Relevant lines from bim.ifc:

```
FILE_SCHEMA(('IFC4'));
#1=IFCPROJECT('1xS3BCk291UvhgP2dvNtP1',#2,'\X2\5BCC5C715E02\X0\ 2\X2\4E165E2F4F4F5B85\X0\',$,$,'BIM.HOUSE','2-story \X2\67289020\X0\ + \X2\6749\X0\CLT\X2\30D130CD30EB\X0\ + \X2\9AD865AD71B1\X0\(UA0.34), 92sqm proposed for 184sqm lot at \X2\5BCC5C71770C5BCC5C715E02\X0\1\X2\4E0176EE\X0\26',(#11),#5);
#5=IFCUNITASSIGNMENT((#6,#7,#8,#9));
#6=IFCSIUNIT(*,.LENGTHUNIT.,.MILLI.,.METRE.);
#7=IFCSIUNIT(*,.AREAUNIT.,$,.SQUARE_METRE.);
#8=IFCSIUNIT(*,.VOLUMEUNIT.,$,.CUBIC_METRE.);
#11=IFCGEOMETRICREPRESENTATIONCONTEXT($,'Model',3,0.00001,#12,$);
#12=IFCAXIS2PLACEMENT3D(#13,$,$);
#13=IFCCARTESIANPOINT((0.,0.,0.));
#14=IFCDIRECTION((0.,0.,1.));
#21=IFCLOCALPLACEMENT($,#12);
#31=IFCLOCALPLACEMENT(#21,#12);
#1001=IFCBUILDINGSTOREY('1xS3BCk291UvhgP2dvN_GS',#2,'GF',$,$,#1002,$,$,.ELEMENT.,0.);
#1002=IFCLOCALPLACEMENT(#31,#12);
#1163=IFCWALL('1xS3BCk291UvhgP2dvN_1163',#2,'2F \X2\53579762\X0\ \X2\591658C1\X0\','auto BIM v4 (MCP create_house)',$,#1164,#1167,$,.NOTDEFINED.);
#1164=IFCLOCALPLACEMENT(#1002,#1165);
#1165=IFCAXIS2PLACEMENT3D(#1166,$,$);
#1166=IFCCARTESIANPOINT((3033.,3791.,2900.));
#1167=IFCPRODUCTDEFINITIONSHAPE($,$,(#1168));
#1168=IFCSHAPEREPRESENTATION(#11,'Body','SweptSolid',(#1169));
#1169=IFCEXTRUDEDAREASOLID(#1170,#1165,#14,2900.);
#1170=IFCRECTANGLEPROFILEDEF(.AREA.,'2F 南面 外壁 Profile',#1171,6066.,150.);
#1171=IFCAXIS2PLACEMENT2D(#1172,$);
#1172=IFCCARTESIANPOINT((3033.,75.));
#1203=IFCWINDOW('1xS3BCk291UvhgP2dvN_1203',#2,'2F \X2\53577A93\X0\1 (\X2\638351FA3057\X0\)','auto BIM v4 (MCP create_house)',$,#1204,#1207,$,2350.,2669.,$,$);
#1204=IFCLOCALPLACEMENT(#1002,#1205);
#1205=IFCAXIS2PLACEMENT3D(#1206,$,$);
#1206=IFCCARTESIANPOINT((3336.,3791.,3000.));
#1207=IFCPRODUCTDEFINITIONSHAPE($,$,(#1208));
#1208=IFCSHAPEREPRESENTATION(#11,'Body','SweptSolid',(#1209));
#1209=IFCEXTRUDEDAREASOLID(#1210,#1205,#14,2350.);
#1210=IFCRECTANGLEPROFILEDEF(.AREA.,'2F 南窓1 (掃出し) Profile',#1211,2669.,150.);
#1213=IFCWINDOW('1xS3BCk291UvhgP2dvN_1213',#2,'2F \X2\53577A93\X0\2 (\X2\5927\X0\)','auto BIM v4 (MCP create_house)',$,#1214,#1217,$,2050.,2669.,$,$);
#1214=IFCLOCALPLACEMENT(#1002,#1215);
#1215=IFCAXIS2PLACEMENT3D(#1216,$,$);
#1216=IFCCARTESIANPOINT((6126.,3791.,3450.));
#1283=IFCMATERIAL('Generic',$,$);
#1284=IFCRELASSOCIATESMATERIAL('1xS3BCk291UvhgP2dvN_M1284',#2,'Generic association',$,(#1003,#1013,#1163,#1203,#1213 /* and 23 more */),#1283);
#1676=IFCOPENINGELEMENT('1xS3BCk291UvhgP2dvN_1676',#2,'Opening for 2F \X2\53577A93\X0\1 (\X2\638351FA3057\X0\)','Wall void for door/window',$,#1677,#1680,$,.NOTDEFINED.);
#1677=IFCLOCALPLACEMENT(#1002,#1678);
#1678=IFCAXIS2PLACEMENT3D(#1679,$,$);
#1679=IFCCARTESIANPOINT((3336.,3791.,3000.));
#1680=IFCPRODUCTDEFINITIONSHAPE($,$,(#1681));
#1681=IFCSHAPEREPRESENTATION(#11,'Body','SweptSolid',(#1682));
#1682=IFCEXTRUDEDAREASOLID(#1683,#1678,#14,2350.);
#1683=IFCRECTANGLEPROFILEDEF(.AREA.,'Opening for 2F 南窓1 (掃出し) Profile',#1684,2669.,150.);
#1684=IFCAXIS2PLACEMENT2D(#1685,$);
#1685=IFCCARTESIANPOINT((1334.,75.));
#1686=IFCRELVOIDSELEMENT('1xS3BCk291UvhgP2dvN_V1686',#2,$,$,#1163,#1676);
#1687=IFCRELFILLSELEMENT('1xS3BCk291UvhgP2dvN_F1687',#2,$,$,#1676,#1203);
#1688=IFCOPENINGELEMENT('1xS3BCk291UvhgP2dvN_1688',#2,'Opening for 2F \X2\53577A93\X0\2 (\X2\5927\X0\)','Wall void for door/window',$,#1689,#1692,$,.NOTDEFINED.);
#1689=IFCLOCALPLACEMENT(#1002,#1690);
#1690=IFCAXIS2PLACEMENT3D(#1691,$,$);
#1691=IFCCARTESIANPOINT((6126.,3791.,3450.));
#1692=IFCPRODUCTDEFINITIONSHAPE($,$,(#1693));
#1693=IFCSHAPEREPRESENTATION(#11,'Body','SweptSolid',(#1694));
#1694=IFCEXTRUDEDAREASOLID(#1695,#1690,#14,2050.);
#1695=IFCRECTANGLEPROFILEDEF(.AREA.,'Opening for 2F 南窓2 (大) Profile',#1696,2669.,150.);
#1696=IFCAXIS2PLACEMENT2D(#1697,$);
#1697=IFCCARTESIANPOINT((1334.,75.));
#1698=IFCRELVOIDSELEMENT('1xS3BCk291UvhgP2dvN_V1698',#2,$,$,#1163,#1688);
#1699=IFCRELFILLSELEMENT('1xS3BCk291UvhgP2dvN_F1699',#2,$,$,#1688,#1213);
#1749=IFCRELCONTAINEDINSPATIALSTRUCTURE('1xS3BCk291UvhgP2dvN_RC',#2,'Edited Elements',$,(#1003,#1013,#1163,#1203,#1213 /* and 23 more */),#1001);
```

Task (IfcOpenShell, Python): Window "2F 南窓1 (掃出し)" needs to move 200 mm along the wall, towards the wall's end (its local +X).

```python
import ifcopenshell
import ifcopenshell.api.geometry
import ifcopenshell.util.placement

model = ifcopenshell.open("bim.ifc")

window = model.by_guid("1xS3BCk291UvhgP2dvN_1203")
opening = window.FillsVoids[0].RelatingOpeningElement
wall = opening.VoidsElements[0].RelatingBuildingElement

wall_matrix = ifcopenshell.util.placement.get_local_placement(wall.ObjectPlacement)
shift = wall_matrix[:3, 0] * 200.0
before = ifcopenshell.util.placement.get_local_placement(window.ObjectPlacement)[:3, 3].copy()

# The window is not placed relative to its opening, so move both.
for product in (opening, window):
    matrix = ifcopenshell.util.placement.get_local_placement(product.ObjectPlacement)
    matrix[:3, 3] += shift
    ifcopenshell.api.geometry.edit_object_placement(model, product=product, matrix=matrix, is_si=False)

after = ifcopenshell.util.placement.get_local_placement(window.ObjectPlacement)[:3, 3]
print("window moved by", (after - before).round(3) + 0.0)

model.write("bim_edited.ifc")
```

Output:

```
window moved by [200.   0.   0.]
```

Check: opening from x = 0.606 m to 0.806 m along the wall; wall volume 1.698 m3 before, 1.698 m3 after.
